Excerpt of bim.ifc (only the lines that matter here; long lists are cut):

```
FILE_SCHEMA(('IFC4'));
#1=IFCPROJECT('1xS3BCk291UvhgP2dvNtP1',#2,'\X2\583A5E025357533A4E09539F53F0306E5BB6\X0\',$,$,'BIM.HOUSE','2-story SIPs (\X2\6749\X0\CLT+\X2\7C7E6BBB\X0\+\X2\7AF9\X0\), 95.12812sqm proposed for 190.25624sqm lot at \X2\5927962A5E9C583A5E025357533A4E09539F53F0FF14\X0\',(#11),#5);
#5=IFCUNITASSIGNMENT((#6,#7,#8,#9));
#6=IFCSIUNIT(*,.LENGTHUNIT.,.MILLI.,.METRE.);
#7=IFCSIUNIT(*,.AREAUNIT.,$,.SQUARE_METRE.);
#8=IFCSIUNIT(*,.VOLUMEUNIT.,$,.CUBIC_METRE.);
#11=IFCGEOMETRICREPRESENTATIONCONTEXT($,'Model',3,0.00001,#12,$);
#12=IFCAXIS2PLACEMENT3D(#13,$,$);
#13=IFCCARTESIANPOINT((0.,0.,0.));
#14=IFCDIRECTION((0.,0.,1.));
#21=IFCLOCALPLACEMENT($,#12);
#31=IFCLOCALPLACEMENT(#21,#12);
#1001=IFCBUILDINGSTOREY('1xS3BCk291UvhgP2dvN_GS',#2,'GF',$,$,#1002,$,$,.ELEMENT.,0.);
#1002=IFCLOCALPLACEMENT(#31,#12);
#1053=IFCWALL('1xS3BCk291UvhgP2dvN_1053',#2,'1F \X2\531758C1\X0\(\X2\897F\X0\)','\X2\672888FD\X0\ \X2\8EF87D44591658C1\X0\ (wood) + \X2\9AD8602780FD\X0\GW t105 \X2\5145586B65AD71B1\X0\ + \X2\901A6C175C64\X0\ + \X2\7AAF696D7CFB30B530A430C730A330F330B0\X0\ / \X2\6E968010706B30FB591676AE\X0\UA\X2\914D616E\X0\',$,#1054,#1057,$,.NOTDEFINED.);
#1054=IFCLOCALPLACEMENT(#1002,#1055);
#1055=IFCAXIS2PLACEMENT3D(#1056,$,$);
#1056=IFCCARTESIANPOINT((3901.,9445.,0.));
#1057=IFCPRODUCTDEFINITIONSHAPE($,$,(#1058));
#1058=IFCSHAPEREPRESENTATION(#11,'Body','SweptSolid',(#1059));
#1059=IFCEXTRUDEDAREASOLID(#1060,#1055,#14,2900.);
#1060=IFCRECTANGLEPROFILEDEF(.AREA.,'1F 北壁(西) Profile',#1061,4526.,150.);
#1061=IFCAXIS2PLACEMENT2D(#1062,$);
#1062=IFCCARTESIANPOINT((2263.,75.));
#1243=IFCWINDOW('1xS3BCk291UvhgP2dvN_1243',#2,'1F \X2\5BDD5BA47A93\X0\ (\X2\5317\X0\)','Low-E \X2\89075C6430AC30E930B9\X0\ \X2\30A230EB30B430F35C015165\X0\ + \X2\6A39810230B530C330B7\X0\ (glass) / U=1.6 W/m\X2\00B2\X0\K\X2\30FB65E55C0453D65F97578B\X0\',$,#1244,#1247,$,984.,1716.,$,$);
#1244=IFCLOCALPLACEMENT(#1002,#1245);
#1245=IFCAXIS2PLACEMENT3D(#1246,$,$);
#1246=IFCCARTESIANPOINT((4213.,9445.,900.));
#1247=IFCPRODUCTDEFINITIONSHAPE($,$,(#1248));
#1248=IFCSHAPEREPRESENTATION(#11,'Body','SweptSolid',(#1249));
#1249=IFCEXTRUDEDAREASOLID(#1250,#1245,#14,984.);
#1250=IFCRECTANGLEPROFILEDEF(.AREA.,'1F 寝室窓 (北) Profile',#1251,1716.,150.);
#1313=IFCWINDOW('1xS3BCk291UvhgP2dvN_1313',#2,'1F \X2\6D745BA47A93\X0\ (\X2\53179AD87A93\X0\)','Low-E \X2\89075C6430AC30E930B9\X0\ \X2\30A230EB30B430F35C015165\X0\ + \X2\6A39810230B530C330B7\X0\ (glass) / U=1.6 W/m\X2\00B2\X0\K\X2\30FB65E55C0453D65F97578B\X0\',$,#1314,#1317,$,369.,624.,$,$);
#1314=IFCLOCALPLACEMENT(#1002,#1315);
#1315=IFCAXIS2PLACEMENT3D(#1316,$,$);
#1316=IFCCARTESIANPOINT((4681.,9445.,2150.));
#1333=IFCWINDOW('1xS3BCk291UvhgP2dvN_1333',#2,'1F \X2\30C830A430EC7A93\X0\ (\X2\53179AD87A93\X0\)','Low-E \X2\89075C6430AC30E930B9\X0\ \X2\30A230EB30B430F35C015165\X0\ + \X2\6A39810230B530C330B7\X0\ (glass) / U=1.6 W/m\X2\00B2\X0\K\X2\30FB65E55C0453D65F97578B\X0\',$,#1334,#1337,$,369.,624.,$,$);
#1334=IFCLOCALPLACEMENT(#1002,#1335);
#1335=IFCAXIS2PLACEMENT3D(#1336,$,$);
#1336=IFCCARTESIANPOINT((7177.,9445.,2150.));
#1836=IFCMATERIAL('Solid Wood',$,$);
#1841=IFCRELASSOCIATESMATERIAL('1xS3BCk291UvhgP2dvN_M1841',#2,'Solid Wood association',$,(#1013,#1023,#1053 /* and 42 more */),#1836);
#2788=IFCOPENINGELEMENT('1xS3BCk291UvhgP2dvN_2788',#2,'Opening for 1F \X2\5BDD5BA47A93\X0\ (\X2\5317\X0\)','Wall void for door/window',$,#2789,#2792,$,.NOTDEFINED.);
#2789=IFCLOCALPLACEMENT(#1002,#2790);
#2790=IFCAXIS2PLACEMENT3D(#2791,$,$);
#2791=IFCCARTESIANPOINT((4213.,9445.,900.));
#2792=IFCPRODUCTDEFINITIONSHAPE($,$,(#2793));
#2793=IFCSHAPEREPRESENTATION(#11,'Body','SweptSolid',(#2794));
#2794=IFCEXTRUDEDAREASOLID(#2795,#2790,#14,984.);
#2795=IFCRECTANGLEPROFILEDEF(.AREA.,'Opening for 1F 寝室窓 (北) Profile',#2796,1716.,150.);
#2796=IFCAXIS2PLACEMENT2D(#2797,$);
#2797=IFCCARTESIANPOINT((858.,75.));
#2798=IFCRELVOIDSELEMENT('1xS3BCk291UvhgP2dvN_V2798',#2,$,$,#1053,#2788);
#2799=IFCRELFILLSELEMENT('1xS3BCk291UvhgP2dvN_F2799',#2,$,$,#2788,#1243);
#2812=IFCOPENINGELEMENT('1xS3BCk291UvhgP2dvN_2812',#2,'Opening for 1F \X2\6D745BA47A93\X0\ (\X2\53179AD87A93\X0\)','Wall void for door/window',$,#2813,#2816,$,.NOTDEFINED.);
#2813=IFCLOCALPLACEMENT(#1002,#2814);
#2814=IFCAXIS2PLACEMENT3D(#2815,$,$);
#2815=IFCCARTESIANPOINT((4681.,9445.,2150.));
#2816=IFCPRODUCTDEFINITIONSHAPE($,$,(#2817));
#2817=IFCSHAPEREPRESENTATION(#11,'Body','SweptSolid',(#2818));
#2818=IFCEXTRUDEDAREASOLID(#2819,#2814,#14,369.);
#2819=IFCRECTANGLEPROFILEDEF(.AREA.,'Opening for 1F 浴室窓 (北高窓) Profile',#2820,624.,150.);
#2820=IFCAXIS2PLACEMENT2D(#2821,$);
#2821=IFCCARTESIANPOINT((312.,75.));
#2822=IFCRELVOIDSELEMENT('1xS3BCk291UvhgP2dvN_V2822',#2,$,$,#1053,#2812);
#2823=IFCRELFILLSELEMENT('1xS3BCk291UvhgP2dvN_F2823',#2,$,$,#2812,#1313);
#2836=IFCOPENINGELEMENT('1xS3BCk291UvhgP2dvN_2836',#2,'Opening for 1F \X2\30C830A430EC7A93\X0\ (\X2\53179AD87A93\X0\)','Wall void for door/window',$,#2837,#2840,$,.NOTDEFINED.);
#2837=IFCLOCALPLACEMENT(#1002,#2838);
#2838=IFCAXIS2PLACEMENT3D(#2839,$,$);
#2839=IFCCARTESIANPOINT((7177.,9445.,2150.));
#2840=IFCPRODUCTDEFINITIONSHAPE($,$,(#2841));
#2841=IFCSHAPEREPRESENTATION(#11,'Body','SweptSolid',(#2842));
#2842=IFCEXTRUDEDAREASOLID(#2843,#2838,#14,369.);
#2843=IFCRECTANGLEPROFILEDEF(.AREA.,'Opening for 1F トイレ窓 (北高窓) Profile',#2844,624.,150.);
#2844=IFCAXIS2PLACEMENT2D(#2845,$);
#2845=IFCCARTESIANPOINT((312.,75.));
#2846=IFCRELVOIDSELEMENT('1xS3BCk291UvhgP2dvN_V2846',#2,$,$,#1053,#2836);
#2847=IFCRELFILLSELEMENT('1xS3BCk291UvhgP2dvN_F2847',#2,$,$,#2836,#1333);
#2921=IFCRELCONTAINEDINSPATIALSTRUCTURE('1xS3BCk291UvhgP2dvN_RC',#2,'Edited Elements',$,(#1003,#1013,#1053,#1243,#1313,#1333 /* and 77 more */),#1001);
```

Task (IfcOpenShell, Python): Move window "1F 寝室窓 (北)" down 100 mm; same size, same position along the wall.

```python
import numpy as np
import ifcopenshell
import ifcopenshell.api.geometry
import ifcopenshell.util.placement
import ifcopenshell.util.unit

model = ifcopenshell.open("bim.ifc")
unit_scale = ifcopenshell.util.unit.calculate_unit_scale(model)

window = model.by_guid("1xS3BCk291UvhgP2dvN_1243")
opening = window.FillsVoids[0].RelatingOpeningElement
dz = -0.1 / unit_scale

shift = np.array([0.0, 0.0, dz])
# The window is not placed relative to its opening, so move both.
for product in (opening, window):
    matrix = ifcopenshell.util.placement.get_local_placement(product.ObjectPlacement)
    matrix[:3, 3] += shift
    ifcopenshell.api.geometry.edit_object_placement(model, product=product, matrix=matrix, is_si=False)

print(f"moved by {dz * unit_scale:+.3f} m")

model.write("bim_rev.ifc")
```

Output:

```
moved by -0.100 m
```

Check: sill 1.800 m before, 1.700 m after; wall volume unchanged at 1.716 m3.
